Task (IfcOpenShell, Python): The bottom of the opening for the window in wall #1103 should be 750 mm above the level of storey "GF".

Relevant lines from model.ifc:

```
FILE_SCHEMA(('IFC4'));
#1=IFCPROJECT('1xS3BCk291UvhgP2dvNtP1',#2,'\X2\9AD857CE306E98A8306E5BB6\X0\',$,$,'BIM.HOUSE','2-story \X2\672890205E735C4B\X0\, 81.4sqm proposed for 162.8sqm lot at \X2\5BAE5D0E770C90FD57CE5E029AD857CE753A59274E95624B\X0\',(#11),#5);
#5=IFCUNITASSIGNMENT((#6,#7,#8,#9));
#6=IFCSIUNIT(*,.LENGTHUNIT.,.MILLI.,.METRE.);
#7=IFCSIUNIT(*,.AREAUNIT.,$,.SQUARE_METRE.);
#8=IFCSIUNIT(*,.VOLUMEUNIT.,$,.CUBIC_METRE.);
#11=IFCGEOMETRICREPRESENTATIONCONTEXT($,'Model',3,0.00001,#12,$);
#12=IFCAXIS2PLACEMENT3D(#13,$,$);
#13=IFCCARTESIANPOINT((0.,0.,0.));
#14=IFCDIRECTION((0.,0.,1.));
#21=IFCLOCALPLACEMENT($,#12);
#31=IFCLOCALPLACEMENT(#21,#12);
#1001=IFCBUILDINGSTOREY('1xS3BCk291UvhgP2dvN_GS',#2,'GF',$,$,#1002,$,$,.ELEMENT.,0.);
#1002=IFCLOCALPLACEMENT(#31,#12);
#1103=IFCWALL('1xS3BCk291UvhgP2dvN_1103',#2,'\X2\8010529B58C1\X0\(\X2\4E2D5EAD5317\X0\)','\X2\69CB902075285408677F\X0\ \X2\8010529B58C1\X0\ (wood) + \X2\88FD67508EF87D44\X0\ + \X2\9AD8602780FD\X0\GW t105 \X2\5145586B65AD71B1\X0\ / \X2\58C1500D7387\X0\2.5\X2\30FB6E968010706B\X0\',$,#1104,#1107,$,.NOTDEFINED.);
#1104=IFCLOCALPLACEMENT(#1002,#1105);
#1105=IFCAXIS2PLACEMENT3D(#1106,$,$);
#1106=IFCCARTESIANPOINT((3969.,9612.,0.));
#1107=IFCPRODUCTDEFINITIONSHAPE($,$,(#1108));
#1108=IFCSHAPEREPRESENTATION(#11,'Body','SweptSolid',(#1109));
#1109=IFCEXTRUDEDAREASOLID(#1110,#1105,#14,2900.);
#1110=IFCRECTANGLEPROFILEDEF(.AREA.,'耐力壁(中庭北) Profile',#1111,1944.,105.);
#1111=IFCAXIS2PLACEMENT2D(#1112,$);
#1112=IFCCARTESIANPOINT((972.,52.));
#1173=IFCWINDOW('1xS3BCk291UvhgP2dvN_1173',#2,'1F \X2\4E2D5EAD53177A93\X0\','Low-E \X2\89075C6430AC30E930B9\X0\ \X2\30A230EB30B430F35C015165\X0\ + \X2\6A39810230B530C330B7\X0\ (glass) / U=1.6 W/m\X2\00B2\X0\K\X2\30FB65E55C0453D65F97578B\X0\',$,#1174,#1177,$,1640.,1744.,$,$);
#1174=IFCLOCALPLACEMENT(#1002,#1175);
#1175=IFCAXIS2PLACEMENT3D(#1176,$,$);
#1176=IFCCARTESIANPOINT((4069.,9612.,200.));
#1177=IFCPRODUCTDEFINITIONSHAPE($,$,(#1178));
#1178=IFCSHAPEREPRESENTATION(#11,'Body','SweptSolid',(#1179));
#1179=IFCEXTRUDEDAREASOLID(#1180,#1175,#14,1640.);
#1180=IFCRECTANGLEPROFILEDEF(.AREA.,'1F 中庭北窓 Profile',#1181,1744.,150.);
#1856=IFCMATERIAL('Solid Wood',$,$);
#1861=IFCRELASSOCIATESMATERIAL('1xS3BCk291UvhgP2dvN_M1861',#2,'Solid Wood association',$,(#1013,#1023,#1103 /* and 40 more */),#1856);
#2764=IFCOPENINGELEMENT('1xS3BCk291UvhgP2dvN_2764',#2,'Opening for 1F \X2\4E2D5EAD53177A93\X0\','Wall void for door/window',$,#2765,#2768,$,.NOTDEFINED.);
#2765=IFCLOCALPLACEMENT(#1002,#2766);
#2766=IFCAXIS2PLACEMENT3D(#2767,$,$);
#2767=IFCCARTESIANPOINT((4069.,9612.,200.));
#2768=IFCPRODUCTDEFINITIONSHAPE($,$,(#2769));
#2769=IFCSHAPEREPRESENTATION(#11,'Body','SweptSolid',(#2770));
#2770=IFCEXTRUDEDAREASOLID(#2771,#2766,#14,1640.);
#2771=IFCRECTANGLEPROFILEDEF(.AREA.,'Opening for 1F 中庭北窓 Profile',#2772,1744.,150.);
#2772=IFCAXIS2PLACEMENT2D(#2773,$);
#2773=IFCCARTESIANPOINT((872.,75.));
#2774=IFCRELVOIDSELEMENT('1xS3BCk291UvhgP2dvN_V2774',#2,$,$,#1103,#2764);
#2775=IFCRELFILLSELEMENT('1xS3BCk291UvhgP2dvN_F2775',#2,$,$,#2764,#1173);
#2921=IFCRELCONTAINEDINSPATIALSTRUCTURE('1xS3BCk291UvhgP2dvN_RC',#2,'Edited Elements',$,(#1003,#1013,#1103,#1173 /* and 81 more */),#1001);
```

```python
import numpy as np
import ifcopenshell
import ifcopenshell.api.geometry
import ifcopenshell.geom
import ifcopenshell.util.element
import ifcopenshell.util.placement
import ifcopenshell.util.shape
import ifcopenshell.util.unit

model = ifcopenshell.open("model.ifc")
unit_scale = ifcopenshell.util.unit.calculate_unit_scale(model)

window = model.by_id(1173)
opening = window.FillsVoids[0].RelatingOpeningElement
storey = ifcopenshell.util.element.get_container(window, ifc_class="IfcBuildingStorey")
level = ifcopenshell.util.placement.get_local_placement(storey.ObjectPlacement)[2, 3]

# The opening's origin need not be at the sill, so measure its lowest point.
shape = ifcopenshell.geom.create_shape(ifcopenshell.geom.settings(), opening)
bottom = ifcopenshell.util.shape.get_shape_bottom_elevation(shape, shape.geometry) / unit_scale
dz = level + 0.75 / unit_scale - bottom

shift = np.array([0.0, 0.0, dz])
# The window is not placed relative to its opening, so move both.
for product in (opening, window):
    matrix = ifcopenshell.util.placement.get_local_placement(product.ObjectPlacement)
    matrix[:3, 3] += shift
    ifcopenshell.api.geometry.edit_object_placement(model, product=product, matrix=matrix, is_si=False)

print(f"moved by {dz * unit_scale:+.3f} m")

model.write("model_v2.ifc")
```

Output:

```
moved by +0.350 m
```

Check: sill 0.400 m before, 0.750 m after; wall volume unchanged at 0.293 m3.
